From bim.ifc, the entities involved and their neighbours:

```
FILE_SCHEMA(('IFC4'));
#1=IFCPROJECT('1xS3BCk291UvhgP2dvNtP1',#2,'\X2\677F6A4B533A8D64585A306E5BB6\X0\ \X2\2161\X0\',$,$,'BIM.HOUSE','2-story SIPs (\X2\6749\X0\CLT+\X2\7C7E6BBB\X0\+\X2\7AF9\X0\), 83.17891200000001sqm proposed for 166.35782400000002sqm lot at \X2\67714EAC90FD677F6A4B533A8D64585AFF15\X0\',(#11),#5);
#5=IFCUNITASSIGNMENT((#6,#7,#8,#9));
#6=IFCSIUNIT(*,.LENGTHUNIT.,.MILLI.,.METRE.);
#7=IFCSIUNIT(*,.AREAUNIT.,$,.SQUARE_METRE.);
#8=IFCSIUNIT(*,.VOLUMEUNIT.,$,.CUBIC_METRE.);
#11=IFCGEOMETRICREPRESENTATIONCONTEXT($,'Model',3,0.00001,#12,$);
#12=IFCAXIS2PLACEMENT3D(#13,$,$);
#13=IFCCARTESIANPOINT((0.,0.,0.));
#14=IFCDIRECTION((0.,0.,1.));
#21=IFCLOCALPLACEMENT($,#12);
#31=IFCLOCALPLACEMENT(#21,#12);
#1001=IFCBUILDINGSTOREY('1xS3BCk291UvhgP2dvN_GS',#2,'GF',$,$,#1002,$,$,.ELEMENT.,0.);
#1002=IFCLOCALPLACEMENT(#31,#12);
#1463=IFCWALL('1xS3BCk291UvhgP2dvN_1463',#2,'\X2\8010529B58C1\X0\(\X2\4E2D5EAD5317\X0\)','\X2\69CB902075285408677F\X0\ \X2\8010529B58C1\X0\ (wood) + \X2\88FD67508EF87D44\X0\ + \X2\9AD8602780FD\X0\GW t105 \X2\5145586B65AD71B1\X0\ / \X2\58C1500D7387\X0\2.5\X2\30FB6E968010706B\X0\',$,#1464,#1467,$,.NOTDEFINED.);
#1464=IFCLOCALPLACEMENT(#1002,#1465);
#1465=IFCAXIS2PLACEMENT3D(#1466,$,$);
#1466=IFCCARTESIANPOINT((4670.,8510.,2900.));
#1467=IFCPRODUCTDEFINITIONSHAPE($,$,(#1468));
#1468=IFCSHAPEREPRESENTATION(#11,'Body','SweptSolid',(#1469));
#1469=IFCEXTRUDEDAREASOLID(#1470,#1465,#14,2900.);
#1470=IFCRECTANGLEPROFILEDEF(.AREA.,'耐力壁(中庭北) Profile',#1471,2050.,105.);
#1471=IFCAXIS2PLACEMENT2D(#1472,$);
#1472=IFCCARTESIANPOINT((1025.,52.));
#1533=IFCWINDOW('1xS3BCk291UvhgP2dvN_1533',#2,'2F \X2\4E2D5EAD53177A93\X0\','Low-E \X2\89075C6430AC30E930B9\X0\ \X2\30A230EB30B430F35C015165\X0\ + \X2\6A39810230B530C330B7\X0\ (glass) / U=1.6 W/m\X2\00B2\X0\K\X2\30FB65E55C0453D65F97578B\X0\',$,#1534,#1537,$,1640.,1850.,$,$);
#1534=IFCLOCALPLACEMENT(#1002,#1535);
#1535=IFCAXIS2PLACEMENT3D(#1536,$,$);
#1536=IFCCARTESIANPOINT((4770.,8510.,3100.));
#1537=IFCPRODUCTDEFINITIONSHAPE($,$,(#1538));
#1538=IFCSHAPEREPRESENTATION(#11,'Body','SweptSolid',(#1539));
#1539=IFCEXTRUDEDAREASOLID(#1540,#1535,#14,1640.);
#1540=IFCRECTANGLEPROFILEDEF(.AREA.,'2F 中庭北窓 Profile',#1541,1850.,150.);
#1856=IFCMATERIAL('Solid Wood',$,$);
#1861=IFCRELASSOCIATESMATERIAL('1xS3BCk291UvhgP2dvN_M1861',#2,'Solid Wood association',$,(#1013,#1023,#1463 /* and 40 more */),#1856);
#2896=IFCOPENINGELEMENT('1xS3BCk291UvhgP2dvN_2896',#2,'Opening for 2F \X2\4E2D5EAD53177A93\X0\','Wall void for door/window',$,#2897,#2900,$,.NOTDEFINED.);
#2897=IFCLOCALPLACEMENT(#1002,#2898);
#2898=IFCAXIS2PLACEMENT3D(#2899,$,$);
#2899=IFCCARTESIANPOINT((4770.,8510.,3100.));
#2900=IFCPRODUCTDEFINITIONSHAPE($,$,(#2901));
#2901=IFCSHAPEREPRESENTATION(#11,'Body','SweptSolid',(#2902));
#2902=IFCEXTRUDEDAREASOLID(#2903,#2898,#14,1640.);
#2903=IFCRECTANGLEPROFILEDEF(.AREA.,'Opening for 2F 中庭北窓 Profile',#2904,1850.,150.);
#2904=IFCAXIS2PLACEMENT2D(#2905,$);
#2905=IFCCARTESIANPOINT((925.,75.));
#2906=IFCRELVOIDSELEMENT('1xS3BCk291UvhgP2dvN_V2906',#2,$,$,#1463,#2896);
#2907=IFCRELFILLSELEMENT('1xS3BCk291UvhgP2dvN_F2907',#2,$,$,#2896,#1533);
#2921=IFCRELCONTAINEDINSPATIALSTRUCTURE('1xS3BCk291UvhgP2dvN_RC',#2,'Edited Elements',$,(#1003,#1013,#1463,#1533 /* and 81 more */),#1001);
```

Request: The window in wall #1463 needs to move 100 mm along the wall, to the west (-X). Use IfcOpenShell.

```python
import ifcopenshell
import ifcopenshell.api.geometry
import ifcopenshell.util.placement

model = ifcopenshell.open("bim.ifc")

window = model.by_guid("1xS3BCk291UvhgP2dvN_1533")
opening = window.FillsVoids[0].RelatingOpeningElement
wall = opening.VoidsElements[0].RelatingBuildingElement

wall_matrix = ifcopenshell.util.placement.get_local_placement(wall.ObjectPlacement)
shift = wall_matrix[:3, 0] * -100.0
before = ifcopenshell.util.placement.get_local_placement(window.ObjectPlacement)[:3, 3].copy()

# The window is not placed relative to its opening, so move both.
for product in (opening, window):
    matrix = ifcopenshell.util.placement.get_local_placement(product.ObjectPlacement)
    matrix[:3, 3] += shift
    ifcopenshell.api.geometry.edit_object_placement(model, product=product, matrix=matrix, is_si=False)

after = ifcopenshell.util.placement.get_local_placement(window.ObjectPlacement)[:3, 3]
print("window moved by", (after - before).round(3) + 0.0)

model.write("bim_rev.ifc")
```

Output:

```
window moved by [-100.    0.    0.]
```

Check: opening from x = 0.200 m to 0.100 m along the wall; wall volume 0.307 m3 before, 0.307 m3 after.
